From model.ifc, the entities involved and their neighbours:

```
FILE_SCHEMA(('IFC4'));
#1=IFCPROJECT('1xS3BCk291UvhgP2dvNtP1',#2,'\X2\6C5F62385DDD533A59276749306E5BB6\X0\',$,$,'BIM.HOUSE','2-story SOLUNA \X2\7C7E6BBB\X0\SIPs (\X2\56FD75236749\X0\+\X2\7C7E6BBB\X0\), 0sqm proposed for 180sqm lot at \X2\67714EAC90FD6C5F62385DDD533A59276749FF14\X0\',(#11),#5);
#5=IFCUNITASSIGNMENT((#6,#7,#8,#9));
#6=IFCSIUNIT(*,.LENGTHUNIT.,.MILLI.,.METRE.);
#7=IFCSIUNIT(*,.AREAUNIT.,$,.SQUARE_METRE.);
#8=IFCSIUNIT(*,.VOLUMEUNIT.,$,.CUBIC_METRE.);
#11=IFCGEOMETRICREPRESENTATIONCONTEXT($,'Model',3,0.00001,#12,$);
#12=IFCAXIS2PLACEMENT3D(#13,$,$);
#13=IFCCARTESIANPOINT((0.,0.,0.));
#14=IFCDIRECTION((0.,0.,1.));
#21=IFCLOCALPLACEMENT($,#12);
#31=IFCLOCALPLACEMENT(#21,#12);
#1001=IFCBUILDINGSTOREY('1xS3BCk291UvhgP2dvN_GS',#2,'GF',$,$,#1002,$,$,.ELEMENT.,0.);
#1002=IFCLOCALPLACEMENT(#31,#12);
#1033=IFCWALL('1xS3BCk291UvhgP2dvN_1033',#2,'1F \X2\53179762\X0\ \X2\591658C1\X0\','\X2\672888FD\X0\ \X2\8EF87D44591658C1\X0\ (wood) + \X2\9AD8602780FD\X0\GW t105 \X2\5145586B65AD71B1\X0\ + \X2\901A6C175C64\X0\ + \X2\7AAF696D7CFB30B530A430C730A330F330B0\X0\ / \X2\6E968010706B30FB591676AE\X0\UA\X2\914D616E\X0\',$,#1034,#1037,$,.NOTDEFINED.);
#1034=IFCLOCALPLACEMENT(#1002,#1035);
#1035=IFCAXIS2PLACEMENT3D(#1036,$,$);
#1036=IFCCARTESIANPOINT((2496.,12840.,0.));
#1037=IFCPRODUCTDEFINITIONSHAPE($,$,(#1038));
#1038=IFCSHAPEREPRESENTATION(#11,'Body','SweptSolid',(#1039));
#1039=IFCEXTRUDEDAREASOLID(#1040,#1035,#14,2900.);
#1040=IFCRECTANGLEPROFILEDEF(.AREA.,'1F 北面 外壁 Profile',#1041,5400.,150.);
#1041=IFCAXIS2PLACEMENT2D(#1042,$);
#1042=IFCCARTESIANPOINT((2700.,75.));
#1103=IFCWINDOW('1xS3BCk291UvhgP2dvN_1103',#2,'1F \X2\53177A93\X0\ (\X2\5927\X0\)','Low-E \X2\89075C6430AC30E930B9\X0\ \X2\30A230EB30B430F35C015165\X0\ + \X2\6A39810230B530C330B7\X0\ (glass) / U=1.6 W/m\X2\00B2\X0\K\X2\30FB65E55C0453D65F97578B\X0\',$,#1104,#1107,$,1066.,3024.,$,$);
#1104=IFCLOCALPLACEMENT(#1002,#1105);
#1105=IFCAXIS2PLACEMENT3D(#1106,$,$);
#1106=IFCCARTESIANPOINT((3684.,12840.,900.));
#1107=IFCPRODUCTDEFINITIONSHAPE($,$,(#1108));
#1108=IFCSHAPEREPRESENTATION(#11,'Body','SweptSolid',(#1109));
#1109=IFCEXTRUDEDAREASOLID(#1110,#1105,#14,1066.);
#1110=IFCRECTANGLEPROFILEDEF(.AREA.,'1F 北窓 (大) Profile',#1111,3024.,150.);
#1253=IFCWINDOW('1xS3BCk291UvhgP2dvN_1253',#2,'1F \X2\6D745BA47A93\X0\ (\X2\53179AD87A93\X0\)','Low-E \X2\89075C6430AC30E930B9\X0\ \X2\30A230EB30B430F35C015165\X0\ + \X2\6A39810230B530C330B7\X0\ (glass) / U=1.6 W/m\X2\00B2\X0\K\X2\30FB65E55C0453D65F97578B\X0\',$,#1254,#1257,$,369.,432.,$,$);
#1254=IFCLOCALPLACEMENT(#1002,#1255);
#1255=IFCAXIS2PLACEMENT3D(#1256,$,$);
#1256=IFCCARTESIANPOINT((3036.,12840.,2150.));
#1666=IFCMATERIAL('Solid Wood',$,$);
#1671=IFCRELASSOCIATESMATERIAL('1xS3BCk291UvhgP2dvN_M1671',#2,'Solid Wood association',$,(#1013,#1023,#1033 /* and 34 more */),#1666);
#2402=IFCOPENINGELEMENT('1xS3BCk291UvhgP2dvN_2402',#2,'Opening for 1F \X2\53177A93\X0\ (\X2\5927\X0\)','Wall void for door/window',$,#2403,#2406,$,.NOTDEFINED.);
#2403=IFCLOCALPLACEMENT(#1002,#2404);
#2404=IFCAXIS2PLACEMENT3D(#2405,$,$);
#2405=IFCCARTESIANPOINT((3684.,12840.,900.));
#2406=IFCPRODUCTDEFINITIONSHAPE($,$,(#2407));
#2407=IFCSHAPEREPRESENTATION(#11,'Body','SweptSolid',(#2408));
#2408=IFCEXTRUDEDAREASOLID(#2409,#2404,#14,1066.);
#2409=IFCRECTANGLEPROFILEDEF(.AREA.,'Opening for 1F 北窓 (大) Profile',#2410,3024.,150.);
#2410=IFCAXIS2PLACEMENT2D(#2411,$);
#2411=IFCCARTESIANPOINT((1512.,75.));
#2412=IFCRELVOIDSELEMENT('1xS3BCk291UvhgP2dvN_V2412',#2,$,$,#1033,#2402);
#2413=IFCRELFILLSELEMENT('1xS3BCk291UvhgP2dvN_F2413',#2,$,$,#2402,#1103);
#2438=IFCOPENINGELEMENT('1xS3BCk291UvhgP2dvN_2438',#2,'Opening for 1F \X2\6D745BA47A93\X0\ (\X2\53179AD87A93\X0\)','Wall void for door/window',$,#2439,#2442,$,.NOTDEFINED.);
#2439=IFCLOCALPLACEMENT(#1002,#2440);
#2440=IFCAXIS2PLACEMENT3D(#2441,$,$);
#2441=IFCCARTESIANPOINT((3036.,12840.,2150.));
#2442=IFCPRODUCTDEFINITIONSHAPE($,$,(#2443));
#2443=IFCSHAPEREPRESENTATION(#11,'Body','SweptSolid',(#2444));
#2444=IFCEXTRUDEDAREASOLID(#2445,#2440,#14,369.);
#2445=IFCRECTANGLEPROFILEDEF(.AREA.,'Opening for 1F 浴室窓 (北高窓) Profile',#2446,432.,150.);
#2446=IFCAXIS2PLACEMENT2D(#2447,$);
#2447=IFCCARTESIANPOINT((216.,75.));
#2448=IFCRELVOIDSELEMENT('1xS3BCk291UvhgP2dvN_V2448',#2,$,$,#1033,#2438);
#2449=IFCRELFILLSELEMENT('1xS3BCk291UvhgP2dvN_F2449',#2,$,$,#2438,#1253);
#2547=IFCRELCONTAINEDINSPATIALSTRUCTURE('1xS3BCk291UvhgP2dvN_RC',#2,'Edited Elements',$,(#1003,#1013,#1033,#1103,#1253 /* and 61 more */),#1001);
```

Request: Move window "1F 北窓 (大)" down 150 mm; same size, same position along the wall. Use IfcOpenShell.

```python
import numpy as np
import ifcopenshell
import ifcopenshell.api.geometry
import ifcopenshell.util.placement
import ifcopenshell.util.unit

model = ifcopenshell.open("model.ifc")
unit_scale = ifcopenshell.util.unit.calculate_unit_scale(model)

window = model.by_id(1103)
opening = window.FillsVoids[0].RelatingOpeningElement
dz = -0.15 / unit_scale

shift = np.array([0.0, 0.0, dz])
# The window is not placed relative to its opening, so move both.
for product in (opening, window):
    matrix = ifcopenshell.util.placement.get_local_placement(product.ObjectPlacement)
    matrix[:3, 3] += shift
    ifcopenshell.api.geometry.edit_object_placement(model, product=product, matrix=matrix, is_si=False)

print(f"moved by {dz * unit_scale:+.3f} m")

model.write("model_updated.ifc")
```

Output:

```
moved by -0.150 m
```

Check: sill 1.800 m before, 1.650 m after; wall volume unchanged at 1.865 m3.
